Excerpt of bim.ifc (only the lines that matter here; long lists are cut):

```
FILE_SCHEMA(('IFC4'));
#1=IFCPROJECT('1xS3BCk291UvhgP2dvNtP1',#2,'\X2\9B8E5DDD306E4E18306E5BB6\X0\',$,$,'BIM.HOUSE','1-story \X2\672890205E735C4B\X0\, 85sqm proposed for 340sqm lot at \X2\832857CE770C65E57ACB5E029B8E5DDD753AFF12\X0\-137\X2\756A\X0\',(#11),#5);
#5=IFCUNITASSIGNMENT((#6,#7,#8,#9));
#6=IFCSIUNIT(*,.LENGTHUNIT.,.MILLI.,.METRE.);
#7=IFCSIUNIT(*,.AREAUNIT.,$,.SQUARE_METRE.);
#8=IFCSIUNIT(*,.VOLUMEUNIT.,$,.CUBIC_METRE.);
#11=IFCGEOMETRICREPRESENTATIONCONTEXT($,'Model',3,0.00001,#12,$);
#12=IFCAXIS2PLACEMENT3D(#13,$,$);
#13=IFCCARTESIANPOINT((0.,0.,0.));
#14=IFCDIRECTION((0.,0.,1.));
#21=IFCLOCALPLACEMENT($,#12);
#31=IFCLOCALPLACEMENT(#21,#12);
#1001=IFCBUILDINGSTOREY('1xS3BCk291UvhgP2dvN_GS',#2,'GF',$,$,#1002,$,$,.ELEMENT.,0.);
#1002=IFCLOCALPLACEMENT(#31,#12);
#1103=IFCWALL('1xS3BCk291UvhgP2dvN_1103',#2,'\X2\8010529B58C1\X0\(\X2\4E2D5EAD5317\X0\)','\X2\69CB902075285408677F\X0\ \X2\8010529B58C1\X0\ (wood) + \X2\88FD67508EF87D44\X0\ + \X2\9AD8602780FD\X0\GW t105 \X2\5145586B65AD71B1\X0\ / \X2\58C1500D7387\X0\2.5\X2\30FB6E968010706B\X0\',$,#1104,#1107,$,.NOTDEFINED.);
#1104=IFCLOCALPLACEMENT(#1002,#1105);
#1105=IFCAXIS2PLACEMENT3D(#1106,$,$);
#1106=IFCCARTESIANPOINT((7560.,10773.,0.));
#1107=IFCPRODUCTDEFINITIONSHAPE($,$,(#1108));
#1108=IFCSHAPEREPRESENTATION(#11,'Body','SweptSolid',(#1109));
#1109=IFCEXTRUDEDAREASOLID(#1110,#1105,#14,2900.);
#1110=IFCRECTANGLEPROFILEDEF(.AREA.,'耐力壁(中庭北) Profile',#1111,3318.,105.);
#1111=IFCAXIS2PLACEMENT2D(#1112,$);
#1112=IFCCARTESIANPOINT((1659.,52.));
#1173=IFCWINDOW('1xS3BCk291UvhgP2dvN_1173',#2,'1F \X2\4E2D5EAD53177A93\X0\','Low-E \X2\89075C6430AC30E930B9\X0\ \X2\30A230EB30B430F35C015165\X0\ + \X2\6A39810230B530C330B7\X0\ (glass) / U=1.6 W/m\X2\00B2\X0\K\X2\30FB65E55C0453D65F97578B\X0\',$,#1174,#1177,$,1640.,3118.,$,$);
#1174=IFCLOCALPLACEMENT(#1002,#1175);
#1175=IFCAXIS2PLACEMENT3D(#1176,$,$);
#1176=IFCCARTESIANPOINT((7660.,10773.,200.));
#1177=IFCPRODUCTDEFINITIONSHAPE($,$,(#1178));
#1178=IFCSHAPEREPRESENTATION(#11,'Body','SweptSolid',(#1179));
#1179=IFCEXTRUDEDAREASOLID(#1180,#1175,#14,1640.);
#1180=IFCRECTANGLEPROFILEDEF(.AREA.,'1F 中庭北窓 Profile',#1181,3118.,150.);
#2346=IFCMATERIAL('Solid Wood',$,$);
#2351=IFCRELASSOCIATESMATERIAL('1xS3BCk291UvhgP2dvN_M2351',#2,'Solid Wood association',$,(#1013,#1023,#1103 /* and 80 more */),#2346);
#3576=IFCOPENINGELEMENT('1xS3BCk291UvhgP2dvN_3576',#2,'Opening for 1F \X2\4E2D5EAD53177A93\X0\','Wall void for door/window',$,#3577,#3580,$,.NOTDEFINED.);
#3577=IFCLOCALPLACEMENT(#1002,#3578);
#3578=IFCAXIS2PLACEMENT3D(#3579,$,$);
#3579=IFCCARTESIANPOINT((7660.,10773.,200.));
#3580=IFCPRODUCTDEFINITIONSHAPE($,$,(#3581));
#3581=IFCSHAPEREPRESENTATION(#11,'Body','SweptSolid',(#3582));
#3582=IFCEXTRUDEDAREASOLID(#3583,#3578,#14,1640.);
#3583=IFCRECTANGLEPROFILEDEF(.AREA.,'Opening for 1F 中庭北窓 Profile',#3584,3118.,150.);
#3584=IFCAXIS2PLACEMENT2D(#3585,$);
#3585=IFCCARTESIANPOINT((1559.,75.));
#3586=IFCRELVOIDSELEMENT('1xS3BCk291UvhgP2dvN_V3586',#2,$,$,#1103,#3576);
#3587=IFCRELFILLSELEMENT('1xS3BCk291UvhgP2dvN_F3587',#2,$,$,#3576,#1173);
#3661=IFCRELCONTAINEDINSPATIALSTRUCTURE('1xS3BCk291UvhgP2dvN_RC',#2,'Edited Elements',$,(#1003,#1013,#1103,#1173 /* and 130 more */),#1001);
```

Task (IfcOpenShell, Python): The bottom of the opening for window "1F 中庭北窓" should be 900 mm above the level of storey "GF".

```python
import numpy as np
import ifcopenshell
import ifcopenshell.api.geometry
import ifcopenshell.geom
import ifcopenshell.util.element
import ifcopenshell.util.placement
import ifcopenshell.util.shape
import ifcopenshell.util.unit

model = ifcopenshell.open("bim.ifc")
unit_scale = ifcopenshell.util.unit.calculate_unit_scale(model)

window = model.by_guid("1xS3BCk291UvhgP2dvN_1173")
opening = window.FillsVoids[0].RelatingOpeningElement
storey = ifcopenshell.util.element.get_container(window, ifc_class="IfcBuildingStorey")
level = ifcopenshell.util.placement.get_local_placement(storey.ObjectPlacement)[2, 3]

# The opening's origin need not be at the sill, so measure its lowest point.
shape = ifcopenshell.geom.create_shape(ifcopenshell.geom.settings(), opening)
bottom = ifcopenshell.util.shape.get_shape_bottom_elevation(shape, shape.geometry) / unit_scale
dz = level + 900.0 - bottom

shift = np.array([0.0, 0.0, dz])
# The window is not placed relative to its opening, so move both.
for product in (opening, window):
    matrix = ifcopenshell.util.placement.get_local_placement(product.ObjectPlacement)
    matrix[:3, 3] += shift
    ifcopenshell.api.geometry.edit_object_placement(model, product=product, matrix=matrix, is_si=False)

print(f"moved by {dz * unit_scale:+.3f} m")

model.write("bim_rev.ifc")
```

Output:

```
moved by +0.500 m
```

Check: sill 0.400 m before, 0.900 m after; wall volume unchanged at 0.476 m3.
